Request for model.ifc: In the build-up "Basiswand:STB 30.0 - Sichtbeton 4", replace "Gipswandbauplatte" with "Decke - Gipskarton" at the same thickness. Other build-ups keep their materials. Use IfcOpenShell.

First a look at what the model holds.

```python
import ifcopenshell
import ifcopenshell.util.element

model = ifcopenshell.open("model.ifc")
print(model.schema)
for layer_set in model.by_type("IfcMaterialLayerSet"):
    if layer_set.LayerSetName == "Basiswand:STB 30.0 - Sichtbeton 4":
        for layer in layer_set.MaterialLayers:
            print(layer.id(), layer.Material and layer.Material.Name, layer.LayerThickness, sep=" | ")
        print(len(ifcopenshell.util.element.get_elements_by_material(model, layer_set)), "elements and types use it")
print(sorted(m.Name for m in model.by_type("IfcMaterial") if m.Name)[:60])
```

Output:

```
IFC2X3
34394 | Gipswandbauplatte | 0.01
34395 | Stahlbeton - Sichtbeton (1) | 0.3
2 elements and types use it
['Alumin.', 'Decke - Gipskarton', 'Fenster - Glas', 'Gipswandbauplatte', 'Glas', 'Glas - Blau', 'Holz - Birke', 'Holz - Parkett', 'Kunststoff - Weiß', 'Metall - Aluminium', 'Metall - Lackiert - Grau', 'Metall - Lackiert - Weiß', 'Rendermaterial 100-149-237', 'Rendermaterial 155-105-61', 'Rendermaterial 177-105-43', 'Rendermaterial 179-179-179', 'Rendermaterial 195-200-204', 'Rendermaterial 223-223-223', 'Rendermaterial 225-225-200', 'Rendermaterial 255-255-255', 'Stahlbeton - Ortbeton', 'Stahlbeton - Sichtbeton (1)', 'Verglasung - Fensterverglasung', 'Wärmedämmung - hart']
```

```python
import ifcopenshell
import ifcopenshell.api.material

model = ifcopenshell.open("model.ifc")

layer_set = next(s for s in model.by_type("IfcMaterialLayerSet") if s.LayerSetName == "Basiswand:STB 30.0 - Sichtbeton 4")
layer = next(l for l in layer_set.MaterialLayers if l.Material and l.Material.Name == "Gipswandbauplatte")
material = next(m for m in model.by_type("IfcMaterial") if m.Name == "Decke - Gipskarton")

# Point this one layer at the other material; renaming the old one would change it everywhere.
ifcopenshell.api.material.edit_layer(model, layer=layer, attributes={}, material=material)

print([l.Material.Name if l.Material else None for l in layer_set.MaterialLayers])

model.write("model-out.ifc")
```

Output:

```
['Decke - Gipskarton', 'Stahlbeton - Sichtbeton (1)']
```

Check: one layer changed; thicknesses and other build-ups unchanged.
